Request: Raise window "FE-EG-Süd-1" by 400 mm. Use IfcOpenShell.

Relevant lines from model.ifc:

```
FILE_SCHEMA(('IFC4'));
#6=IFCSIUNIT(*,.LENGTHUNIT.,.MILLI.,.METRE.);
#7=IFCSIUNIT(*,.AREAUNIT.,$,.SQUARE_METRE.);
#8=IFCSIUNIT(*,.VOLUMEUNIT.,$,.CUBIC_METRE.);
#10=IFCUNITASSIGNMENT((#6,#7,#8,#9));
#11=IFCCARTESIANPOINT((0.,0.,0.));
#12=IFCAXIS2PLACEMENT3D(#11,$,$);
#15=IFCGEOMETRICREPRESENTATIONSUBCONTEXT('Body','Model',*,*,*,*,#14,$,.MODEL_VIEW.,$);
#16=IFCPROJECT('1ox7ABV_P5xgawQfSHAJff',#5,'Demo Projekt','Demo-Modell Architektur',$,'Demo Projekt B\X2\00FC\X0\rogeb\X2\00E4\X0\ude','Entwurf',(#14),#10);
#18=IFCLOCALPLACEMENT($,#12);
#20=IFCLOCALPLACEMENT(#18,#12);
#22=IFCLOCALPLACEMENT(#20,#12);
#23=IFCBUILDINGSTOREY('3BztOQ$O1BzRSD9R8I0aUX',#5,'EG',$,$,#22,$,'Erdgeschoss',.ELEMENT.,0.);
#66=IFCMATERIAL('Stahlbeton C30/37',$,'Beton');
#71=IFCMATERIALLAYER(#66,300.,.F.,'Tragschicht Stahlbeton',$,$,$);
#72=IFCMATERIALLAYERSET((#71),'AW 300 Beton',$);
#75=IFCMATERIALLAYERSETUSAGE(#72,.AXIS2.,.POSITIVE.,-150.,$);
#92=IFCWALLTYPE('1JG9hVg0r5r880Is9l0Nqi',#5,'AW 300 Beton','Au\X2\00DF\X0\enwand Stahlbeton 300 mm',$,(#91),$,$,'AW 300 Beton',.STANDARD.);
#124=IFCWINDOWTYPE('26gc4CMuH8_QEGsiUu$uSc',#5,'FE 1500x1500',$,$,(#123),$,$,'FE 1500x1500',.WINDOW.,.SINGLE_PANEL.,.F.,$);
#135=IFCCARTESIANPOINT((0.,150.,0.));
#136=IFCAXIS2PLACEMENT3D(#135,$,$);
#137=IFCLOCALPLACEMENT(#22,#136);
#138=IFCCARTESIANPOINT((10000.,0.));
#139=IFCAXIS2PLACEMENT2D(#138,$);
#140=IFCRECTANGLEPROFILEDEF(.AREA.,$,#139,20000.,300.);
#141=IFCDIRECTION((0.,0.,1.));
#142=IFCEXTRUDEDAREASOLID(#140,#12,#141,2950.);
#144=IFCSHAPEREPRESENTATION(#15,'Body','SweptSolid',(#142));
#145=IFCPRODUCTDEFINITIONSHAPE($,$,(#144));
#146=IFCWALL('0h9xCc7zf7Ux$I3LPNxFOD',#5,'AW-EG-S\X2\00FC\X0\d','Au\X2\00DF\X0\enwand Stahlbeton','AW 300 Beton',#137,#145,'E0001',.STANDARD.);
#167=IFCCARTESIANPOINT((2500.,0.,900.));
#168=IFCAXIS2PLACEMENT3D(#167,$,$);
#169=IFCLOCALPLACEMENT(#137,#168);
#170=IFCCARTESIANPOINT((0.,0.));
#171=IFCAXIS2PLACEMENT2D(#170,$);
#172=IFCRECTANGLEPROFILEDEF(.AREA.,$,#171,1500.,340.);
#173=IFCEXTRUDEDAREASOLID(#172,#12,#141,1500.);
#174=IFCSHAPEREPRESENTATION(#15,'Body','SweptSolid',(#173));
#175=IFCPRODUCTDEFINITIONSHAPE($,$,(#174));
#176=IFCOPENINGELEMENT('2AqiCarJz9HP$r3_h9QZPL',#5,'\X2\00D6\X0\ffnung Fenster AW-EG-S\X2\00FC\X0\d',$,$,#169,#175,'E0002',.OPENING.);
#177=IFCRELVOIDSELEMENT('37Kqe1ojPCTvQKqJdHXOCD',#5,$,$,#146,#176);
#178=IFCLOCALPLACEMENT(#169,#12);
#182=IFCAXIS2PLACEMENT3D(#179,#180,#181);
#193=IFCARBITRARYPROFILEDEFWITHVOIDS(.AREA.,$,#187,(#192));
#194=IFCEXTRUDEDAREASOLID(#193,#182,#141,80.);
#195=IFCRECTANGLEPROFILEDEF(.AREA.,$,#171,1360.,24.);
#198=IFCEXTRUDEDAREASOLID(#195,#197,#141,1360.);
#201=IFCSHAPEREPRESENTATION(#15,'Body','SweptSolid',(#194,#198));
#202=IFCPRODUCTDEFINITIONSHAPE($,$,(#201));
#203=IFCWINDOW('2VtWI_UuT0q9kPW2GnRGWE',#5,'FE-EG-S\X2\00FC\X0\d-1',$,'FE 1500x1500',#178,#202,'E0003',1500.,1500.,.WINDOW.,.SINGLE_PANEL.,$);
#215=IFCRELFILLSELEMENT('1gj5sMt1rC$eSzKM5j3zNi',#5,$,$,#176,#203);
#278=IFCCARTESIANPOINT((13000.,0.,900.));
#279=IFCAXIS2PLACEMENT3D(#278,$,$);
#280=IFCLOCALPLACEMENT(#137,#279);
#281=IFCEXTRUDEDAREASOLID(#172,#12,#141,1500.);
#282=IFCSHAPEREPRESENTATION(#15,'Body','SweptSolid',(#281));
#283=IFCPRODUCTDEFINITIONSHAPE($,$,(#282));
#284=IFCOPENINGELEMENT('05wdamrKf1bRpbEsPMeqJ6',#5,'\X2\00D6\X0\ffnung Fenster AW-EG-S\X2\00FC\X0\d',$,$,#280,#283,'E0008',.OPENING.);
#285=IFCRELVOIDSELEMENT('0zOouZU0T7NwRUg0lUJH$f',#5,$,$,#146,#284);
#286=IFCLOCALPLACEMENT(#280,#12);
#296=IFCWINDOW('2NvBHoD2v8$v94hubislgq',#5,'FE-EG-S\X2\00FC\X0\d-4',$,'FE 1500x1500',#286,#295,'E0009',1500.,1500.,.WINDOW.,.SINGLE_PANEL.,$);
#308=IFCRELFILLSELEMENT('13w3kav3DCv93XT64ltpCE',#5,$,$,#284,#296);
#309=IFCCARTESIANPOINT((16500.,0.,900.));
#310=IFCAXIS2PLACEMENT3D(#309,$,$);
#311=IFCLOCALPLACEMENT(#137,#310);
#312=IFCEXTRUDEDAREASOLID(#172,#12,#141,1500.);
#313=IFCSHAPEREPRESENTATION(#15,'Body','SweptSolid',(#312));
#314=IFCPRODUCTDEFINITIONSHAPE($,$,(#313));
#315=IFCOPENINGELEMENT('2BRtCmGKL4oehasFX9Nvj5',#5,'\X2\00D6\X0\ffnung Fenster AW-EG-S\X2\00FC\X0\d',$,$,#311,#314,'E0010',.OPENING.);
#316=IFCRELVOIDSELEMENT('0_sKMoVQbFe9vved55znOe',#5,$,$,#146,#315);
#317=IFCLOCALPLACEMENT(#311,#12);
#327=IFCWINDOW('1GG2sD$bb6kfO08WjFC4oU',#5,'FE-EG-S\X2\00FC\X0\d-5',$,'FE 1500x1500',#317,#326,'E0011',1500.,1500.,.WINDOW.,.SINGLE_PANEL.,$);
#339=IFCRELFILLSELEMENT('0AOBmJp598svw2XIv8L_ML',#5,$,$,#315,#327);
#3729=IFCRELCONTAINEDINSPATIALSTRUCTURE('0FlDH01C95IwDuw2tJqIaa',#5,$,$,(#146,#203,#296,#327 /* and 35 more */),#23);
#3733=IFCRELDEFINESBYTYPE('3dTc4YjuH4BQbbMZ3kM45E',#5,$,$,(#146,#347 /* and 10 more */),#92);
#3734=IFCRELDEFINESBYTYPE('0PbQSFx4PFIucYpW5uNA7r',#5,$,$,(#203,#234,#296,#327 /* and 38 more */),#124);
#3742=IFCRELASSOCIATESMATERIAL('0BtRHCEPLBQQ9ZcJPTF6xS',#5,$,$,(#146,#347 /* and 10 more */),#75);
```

```python
import numpy as np
import ifcopenshell
import ifcopenshell.api.geometry
import ifcopenshell.util.placement
import ifcopenshell.util.unit

model = ifcopenshell.open("model.ifc")
unit_scale = ifcopenshell.util.unit.calculate_unit_scale(model)

window = model.by_guid("2VtWI_UuT0q9kPW2GnRGWE")
opening = window.FillsVoids[0].RelatingOpeningElement
dz = 0.4 / unit_scale

shift = np.array([0.0, 0.0, dz])
# The window is placed relative to its opening, so it follows when the opening moves.
matrix = ifcopenshell.util.placement.get_local_placement(opening.ObjectPlacement)
matrix[:3, 3] += shift
ifcopenshell.api.geometry.edit_object_placement(
    model, product=opening, matrix=matrix, is_si=False, should_transform_children=True
)

print(f"moved by {dz * unit_scale:+.3f} m")

model.write("model_edited.ifc")
```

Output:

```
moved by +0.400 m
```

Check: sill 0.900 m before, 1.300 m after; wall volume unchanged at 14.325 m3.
